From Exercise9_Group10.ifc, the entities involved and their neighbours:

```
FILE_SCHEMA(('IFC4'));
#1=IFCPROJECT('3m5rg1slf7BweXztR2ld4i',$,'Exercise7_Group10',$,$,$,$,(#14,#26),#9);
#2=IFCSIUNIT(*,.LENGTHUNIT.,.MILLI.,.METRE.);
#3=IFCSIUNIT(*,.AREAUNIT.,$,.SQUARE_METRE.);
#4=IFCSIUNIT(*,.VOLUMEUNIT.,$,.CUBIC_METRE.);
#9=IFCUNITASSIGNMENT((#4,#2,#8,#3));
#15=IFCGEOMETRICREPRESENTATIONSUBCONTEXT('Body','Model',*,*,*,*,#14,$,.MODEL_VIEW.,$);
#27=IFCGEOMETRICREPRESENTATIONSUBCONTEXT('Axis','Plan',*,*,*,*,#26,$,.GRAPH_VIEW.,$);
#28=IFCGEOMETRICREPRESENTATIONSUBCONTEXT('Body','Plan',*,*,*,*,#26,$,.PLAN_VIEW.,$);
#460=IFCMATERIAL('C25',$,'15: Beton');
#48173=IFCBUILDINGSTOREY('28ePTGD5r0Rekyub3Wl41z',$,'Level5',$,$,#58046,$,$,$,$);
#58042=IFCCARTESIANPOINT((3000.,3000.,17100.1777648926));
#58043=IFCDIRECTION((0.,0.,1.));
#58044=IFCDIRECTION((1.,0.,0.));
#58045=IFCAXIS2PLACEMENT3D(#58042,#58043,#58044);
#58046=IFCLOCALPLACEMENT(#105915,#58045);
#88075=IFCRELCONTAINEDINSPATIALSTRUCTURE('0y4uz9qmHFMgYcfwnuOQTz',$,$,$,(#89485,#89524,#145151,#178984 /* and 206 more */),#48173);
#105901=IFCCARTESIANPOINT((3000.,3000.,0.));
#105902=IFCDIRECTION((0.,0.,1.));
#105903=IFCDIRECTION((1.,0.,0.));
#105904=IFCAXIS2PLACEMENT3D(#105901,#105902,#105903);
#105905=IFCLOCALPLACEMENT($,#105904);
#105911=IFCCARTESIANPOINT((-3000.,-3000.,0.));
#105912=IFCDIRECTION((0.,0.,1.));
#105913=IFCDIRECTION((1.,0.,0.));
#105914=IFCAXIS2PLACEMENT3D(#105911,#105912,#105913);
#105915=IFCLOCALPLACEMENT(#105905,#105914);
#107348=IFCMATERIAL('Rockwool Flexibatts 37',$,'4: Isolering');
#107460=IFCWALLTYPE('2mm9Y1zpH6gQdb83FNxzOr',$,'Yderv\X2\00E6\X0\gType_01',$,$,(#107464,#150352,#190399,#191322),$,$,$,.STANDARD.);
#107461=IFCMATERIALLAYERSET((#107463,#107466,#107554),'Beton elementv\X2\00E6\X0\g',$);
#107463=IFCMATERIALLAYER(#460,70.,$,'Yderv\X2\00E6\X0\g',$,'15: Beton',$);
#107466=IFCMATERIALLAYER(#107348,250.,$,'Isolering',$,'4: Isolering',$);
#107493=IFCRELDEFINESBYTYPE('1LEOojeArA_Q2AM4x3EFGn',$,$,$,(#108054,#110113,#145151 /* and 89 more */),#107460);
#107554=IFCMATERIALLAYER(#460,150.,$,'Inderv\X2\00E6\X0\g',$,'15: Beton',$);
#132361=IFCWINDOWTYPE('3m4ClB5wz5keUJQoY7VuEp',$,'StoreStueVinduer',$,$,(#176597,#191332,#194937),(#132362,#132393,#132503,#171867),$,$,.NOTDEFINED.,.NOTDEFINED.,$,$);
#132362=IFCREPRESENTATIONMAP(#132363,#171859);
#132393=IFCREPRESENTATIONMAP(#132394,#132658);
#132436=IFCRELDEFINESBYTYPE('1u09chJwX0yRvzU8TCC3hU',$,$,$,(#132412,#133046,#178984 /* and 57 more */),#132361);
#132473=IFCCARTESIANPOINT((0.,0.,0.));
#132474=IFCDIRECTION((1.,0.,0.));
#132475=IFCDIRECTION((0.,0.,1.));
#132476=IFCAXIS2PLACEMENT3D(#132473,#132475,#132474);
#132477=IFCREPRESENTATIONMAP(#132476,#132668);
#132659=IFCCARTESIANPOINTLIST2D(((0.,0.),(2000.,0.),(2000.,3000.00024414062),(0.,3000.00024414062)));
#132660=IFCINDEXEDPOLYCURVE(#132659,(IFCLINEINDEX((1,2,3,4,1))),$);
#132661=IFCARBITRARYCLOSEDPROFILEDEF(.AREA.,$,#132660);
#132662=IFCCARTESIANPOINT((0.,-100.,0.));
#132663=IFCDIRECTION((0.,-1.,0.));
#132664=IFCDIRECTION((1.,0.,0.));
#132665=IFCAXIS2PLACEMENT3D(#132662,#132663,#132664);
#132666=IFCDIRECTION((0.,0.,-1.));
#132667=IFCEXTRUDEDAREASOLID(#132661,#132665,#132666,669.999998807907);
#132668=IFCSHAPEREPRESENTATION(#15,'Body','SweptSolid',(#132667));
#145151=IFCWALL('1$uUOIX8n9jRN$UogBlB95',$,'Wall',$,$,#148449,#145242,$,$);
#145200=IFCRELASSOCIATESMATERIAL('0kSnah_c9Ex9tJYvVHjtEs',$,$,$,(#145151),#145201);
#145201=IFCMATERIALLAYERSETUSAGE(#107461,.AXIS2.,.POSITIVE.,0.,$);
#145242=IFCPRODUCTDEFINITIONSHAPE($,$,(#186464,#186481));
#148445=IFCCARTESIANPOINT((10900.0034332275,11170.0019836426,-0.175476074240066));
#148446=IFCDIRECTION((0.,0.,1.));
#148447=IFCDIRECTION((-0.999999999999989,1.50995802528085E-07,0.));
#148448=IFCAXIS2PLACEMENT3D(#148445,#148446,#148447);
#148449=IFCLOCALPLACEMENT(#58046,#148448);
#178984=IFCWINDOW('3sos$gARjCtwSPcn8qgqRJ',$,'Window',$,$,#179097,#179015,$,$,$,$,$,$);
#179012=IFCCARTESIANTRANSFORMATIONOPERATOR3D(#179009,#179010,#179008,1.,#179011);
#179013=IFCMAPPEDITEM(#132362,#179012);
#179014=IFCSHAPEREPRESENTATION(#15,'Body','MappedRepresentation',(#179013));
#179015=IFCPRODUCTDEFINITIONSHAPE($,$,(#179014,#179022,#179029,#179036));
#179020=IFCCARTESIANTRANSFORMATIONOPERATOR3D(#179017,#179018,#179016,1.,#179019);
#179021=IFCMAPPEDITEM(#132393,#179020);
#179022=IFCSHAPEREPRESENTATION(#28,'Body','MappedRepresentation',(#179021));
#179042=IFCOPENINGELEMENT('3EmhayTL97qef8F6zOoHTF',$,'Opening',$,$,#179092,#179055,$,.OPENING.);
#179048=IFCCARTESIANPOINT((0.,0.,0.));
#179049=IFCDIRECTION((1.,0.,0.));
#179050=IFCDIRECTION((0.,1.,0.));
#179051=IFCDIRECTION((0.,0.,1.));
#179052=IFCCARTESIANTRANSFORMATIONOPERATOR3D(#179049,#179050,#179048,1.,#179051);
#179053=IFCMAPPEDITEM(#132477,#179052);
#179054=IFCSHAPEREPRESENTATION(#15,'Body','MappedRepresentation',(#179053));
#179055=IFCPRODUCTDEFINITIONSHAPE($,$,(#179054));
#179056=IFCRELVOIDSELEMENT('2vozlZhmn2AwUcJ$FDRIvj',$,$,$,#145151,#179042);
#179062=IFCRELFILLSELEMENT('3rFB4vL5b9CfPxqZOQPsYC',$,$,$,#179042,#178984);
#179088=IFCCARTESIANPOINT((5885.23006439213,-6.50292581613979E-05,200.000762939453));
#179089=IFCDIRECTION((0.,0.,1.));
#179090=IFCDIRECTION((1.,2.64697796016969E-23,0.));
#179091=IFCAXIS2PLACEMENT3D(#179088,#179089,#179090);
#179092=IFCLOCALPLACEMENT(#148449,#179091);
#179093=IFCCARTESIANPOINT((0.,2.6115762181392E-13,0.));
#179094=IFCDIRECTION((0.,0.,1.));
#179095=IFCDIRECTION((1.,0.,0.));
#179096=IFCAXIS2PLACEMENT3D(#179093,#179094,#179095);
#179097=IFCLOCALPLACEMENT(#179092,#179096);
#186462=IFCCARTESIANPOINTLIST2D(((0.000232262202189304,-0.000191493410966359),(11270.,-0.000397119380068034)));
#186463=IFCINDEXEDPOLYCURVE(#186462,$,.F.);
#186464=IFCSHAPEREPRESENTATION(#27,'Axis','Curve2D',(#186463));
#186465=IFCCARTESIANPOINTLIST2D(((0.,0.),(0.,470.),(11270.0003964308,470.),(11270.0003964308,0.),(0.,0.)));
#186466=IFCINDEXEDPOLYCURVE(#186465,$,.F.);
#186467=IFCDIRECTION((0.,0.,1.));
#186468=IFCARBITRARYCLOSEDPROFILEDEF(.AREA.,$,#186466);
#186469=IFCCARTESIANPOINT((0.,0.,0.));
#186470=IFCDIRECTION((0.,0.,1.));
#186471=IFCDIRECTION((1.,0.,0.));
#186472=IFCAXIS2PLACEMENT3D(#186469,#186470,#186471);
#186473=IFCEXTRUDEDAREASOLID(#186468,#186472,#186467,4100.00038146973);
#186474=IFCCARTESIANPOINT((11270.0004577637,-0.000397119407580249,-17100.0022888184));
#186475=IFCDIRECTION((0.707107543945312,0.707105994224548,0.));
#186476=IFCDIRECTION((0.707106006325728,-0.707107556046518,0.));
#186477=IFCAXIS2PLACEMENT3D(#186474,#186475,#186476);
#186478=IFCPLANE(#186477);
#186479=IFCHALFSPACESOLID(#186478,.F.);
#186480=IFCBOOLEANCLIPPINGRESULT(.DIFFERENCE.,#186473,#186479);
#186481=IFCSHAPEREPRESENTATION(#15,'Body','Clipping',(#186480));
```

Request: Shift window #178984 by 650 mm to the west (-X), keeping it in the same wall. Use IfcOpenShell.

```python
import ifcopenshell
import ifcopenshell.api.geometry
import ifcopenshell.util.placement
import ifcopenshell.util.unit

model = ifcopenshell.open("Exercise9_Group10.ifc")
unit_scale = ifcopenshell.util.unit.calculate_unit_scale(model)

window = model.by_id(178984)
opening = window.FillsVoids[0].RelatingOpeningElement
wall = opening.VoidsElements[0].RelatingBuildingElement

wall_matrix = ifcopenshell.util.placement.get_local_placement(wall.ObjectPlacement)
shift = wall_matrix[:3, 0] * 0.65 / unit_scale
before = ifcopenshell.util.placement.get_local_placement(window.ObjectPlacement)[:3, 3].copy()

# The window is placed relative to its opening, so it follows when the opening moves.
matrix = ifcopenshell.util.placement.get_local_placement(opening.ObjectPlacement)
matrix[:3, 3] += shift
ifcopenshell.api.geometry.edit_object_placement(
    model, product=opening, matrix=matrix, is_si=False, should_transform_children=True
)

after = ifcopenshell.util.placement.get_local_placement(window.ObjectPlacement)[:3, 3]
print("window moved by", (after - before).round(3) + 0.0)

model.write("Exercise9_Group10-out.ifc")
```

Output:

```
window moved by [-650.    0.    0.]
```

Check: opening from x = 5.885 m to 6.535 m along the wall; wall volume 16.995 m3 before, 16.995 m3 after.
